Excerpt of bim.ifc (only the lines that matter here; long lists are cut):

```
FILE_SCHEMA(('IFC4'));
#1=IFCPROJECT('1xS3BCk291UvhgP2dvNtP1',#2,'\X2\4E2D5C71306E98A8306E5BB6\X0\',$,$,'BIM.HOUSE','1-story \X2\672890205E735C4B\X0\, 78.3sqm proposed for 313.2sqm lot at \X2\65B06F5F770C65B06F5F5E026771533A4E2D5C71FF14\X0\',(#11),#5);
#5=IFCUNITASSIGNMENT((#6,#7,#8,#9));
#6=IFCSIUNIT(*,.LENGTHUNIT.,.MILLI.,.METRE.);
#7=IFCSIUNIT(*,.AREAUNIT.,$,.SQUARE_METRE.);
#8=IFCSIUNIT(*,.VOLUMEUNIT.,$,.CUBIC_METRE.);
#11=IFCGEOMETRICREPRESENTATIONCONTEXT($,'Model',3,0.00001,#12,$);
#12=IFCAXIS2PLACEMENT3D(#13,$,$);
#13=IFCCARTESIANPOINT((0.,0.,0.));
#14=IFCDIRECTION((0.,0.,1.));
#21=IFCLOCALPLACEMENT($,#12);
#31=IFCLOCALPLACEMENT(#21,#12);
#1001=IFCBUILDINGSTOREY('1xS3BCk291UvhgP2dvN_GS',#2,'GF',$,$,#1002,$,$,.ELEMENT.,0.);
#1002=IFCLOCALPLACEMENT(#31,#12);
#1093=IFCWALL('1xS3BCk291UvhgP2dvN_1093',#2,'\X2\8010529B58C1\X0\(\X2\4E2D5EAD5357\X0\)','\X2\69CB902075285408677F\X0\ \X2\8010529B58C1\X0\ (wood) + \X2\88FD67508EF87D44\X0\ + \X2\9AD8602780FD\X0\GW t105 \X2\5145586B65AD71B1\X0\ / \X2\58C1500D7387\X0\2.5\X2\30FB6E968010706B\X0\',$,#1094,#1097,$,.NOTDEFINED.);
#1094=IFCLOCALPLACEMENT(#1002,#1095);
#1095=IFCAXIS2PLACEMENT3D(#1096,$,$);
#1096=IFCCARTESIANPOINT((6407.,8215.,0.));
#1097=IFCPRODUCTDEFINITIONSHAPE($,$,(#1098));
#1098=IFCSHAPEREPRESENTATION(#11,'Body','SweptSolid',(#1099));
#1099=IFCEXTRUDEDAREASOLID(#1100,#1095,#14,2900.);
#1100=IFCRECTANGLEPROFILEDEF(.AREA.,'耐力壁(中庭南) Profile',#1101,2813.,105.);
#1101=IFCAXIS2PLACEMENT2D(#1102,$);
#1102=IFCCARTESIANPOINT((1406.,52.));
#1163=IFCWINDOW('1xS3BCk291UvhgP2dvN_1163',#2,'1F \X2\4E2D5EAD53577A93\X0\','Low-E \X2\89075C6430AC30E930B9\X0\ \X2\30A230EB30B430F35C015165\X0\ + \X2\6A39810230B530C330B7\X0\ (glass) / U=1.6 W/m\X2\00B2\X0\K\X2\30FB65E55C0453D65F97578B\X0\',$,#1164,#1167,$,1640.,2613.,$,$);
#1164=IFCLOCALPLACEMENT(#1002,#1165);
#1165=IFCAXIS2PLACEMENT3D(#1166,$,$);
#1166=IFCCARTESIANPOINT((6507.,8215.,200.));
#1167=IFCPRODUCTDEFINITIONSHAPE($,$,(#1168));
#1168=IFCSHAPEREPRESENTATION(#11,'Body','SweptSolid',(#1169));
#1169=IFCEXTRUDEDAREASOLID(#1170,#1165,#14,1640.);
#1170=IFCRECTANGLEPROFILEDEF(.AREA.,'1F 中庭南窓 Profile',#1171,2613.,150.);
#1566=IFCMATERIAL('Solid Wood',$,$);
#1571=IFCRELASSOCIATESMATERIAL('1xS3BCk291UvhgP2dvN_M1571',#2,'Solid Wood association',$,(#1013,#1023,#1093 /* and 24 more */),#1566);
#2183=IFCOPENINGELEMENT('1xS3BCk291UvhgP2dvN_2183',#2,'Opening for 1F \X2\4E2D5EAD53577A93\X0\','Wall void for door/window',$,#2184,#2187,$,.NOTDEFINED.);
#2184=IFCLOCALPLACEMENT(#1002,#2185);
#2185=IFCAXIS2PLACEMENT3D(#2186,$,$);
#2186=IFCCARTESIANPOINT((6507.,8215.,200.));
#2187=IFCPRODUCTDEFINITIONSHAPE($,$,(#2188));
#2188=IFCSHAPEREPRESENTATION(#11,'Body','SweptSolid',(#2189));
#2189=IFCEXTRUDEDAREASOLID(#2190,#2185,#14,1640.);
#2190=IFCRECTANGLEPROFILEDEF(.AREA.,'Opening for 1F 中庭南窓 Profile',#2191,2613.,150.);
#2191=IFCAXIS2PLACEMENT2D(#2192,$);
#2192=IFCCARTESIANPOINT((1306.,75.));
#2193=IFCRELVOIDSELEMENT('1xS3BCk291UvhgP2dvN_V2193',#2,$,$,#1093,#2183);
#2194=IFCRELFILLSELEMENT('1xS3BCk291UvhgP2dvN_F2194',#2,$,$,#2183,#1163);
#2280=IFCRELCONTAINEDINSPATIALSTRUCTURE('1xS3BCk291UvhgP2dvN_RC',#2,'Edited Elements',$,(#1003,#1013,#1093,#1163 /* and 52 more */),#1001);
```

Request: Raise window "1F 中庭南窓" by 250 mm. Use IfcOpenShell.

```python
import numpy as np
import ifcopenshell
import ifcopenshell.api.geometry
import ifcopenshell.util.placement
import ifcopenshell.util.unit

model = ifcopenshell.open("bim.ifc")
unit_scale = ifcopenshell.util.unit.calculate_unit_scale(model)

window = model.by_guid("1xS3BCk291UvhgP2dvN_1163")
opening = window.FillsVoids[0].RelatingOpeningElement
dz = 250.0

shift = np.array([0.0, 0.0, dz])
# The window is not placed relative to its opening, so move both.
for product in (opening, window):
    matrix = ifcopenshell.util.placement.get_local_placement(product.ObjectPlacement)
    matrix[:3, 3] += shift
    ifcopenshell.api.geometry.edit_object_placement(model, product=product, matrix=matrix, is_si=False)

print(f"moved by {dz * unit_scale:+.3f} m")

model.write("bim_updated.ifc")
```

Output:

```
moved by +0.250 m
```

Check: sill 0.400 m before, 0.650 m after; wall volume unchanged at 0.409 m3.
